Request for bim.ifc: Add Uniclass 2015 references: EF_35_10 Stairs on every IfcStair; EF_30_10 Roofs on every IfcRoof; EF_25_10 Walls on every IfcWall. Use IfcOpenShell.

First a look at what the model holds.

```python
import ifcopenshell

model = ifcopenshell.open("bim.ifc")
print(model.schema)
print("classifications:", [c.Name for c in model.by_type("IfcClassification")])
for ifc_class in ("IfcDoor", "IfcRoof", "IfcStair", "IfcWall", "IfcWindow"):
    print(ifc_class, len(model.by_type(ifc_class)))
```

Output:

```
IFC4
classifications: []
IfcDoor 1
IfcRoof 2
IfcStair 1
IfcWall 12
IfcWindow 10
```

```python
import ifcopenshell
import ifcopenshell.api.classification

model = ifcopenshell.open("bim.ifc")

system = ifcopenshell.api.classification.add_classification(model, classification="Uniclass 2015")

codes = {
    "IfcStair": ("EF_35_10", "Stairs"),
    "IfcRoof": ("EF_30_10", "Roofs"),
    "IfcWall": ("EF_25_10", "Walls"),
}
for ifc_class, (code, name) in codes.items():
    products = model.by_type(ifc_class)
    ifcopenshell.api.classification.add_reference(
        model, products=products, classification=system, identification=code, name=name
    )
    print(code, len(products))

model.write("bim_rev.ifc")
```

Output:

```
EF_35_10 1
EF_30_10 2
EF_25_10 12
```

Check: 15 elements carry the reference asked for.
